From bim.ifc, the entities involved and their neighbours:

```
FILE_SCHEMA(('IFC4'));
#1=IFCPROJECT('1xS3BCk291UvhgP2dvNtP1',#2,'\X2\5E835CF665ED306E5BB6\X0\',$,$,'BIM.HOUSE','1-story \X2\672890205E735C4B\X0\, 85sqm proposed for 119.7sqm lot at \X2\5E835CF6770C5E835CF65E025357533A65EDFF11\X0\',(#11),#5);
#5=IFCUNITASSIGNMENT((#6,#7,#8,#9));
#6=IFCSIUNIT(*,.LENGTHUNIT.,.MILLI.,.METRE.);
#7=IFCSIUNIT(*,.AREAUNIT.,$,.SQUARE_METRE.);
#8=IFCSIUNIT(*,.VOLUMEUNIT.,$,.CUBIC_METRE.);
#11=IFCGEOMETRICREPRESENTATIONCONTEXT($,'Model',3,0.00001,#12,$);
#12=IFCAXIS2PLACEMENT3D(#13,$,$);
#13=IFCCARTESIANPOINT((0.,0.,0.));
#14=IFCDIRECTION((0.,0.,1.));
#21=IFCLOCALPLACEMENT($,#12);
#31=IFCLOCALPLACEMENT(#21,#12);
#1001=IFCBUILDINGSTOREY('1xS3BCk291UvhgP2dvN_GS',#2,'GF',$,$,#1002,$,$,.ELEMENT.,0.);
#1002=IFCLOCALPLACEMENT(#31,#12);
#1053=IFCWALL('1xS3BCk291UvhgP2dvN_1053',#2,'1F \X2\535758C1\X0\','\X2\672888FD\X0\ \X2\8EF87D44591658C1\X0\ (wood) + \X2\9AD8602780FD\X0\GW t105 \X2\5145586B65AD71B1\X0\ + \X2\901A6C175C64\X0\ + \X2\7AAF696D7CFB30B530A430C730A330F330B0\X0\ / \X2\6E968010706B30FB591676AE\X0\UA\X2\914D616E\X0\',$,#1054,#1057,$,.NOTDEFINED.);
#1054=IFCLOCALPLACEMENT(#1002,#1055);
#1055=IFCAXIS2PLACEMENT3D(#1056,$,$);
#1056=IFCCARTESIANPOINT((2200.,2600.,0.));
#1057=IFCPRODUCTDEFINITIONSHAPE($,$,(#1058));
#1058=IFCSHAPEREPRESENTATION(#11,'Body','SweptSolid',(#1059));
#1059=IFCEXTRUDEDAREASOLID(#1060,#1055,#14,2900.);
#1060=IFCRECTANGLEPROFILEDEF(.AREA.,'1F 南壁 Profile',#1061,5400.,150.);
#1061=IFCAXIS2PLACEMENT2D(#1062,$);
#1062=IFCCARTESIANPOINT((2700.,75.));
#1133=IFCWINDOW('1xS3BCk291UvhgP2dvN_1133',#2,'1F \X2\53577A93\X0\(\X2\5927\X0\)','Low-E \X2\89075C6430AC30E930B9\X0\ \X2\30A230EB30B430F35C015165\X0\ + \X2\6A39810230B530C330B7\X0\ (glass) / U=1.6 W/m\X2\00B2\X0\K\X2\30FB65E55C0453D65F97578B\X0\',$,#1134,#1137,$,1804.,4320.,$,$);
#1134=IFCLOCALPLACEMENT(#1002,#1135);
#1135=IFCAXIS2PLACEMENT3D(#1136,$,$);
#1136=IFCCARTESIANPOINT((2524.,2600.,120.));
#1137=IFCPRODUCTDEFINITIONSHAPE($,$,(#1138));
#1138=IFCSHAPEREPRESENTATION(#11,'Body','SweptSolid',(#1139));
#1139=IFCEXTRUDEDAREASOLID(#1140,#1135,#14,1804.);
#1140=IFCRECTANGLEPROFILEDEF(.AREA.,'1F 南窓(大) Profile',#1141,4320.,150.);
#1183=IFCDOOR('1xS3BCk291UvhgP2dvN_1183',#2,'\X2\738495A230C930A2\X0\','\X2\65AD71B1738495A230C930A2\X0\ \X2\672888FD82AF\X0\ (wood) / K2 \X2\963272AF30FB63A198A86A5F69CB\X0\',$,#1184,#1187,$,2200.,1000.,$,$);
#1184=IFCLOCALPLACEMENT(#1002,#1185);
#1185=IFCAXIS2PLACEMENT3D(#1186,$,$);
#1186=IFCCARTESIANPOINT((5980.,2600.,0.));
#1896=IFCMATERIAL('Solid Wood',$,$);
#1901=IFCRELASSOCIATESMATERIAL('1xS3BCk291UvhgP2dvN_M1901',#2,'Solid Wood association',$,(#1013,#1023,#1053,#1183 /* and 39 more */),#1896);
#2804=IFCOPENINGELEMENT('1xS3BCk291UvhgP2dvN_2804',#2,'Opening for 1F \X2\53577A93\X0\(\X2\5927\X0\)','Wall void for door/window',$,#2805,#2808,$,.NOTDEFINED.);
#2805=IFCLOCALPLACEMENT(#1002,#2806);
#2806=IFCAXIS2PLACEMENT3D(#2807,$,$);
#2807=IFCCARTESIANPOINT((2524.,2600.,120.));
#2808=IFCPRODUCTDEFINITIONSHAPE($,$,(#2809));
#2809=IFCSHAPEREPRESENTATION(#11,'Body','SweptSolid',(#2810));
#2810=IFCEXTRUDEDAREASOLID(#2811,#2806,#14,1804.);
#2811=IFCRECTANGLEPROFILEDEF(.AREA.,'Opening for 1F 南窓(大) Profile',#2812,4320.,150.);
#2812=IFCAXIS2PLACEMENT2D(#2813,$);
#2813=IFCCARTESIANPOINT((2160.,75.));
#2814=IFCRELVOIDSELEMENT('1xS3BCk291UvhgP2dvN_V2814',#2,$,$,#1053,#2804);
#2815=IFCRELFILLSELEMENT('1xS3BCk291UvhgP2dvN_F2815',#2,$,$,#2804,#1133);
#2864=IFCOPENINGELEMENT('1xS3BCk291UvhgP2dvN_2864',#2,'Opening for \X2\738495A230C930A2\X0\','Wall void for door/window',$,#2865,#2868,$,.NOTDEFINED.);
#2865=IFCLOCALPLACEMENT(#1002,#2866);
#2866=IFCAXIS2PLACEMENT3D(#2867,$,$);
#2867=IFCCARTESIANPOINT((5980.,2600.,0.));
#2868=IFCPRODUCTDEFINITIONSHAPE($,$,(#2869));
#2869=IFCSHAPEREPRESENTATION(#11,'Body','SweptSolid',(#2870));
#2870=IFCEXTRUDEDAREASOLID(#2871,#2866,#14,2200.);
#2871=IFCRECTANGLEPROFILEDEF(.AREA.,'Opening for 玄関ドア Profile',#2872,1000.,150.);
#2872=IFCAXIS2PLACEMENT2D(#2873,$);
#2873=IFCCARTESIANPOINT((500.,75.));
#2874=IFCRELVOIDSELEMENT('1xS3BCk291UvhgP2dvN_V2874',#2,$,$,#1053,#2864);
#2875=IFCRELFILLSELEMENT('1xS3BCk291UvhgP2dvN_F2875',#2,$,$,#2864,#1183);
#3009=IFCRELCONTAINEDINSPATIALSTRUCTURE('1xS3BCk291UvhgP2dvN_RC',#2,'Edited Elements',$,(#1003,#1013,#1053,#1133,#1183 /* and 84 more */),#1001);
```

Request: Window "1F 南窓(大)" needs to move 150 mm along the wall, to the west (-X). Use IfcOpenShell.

```python
import ifcopenshell
import ifcopenshell.api.geometry
import ifcopenshell.util.placement
import ifcopenshell.util.unit

model = ifcopenshell.open("bim.ifc")
unit_scale = ifcopenshell.util.unit.calculate_unit_scale(model)

window = model.by_guid("1xS3BCk291UvhgP2dvN_1133")
opening = window.FillsVoids[0].RelatingOpeningElement
wall = opening.VoidsElements[0].RelatingBuildingElement

wall_matrix = ifcopenshell.util.placement.get_local_placement(wall.ObjectPlacement)
shift = wall_matrix[:3, 0] * -0.15 / unit_scale
before = ifcopenshell.util.placement.get_local_placement(window.ObjectPlacement)[:3, 3].copy()

# The window is not placed relative to its opening, so move both.
for product in (opening, window):
    matrix = ifcopenshell.util.placement.get_local_placement(product.ObjectPlacement)
    matrix[:3, 3] += shift
    ifcopenshell.api.geometry.edit_object_placement(model, product=product, matrix=matrix, is_si=False)

after = ifcopenshell.util.placement.get_local_placement(window.ObjectPlacement)[:3, 3]
print("window moved by", (after - before).round(3) + 0.0)

model.write("bim_v2.ifc")
```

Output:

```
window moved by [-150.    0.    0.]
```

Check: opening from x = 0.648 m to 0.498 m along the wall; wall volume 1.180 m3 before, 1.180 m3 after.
